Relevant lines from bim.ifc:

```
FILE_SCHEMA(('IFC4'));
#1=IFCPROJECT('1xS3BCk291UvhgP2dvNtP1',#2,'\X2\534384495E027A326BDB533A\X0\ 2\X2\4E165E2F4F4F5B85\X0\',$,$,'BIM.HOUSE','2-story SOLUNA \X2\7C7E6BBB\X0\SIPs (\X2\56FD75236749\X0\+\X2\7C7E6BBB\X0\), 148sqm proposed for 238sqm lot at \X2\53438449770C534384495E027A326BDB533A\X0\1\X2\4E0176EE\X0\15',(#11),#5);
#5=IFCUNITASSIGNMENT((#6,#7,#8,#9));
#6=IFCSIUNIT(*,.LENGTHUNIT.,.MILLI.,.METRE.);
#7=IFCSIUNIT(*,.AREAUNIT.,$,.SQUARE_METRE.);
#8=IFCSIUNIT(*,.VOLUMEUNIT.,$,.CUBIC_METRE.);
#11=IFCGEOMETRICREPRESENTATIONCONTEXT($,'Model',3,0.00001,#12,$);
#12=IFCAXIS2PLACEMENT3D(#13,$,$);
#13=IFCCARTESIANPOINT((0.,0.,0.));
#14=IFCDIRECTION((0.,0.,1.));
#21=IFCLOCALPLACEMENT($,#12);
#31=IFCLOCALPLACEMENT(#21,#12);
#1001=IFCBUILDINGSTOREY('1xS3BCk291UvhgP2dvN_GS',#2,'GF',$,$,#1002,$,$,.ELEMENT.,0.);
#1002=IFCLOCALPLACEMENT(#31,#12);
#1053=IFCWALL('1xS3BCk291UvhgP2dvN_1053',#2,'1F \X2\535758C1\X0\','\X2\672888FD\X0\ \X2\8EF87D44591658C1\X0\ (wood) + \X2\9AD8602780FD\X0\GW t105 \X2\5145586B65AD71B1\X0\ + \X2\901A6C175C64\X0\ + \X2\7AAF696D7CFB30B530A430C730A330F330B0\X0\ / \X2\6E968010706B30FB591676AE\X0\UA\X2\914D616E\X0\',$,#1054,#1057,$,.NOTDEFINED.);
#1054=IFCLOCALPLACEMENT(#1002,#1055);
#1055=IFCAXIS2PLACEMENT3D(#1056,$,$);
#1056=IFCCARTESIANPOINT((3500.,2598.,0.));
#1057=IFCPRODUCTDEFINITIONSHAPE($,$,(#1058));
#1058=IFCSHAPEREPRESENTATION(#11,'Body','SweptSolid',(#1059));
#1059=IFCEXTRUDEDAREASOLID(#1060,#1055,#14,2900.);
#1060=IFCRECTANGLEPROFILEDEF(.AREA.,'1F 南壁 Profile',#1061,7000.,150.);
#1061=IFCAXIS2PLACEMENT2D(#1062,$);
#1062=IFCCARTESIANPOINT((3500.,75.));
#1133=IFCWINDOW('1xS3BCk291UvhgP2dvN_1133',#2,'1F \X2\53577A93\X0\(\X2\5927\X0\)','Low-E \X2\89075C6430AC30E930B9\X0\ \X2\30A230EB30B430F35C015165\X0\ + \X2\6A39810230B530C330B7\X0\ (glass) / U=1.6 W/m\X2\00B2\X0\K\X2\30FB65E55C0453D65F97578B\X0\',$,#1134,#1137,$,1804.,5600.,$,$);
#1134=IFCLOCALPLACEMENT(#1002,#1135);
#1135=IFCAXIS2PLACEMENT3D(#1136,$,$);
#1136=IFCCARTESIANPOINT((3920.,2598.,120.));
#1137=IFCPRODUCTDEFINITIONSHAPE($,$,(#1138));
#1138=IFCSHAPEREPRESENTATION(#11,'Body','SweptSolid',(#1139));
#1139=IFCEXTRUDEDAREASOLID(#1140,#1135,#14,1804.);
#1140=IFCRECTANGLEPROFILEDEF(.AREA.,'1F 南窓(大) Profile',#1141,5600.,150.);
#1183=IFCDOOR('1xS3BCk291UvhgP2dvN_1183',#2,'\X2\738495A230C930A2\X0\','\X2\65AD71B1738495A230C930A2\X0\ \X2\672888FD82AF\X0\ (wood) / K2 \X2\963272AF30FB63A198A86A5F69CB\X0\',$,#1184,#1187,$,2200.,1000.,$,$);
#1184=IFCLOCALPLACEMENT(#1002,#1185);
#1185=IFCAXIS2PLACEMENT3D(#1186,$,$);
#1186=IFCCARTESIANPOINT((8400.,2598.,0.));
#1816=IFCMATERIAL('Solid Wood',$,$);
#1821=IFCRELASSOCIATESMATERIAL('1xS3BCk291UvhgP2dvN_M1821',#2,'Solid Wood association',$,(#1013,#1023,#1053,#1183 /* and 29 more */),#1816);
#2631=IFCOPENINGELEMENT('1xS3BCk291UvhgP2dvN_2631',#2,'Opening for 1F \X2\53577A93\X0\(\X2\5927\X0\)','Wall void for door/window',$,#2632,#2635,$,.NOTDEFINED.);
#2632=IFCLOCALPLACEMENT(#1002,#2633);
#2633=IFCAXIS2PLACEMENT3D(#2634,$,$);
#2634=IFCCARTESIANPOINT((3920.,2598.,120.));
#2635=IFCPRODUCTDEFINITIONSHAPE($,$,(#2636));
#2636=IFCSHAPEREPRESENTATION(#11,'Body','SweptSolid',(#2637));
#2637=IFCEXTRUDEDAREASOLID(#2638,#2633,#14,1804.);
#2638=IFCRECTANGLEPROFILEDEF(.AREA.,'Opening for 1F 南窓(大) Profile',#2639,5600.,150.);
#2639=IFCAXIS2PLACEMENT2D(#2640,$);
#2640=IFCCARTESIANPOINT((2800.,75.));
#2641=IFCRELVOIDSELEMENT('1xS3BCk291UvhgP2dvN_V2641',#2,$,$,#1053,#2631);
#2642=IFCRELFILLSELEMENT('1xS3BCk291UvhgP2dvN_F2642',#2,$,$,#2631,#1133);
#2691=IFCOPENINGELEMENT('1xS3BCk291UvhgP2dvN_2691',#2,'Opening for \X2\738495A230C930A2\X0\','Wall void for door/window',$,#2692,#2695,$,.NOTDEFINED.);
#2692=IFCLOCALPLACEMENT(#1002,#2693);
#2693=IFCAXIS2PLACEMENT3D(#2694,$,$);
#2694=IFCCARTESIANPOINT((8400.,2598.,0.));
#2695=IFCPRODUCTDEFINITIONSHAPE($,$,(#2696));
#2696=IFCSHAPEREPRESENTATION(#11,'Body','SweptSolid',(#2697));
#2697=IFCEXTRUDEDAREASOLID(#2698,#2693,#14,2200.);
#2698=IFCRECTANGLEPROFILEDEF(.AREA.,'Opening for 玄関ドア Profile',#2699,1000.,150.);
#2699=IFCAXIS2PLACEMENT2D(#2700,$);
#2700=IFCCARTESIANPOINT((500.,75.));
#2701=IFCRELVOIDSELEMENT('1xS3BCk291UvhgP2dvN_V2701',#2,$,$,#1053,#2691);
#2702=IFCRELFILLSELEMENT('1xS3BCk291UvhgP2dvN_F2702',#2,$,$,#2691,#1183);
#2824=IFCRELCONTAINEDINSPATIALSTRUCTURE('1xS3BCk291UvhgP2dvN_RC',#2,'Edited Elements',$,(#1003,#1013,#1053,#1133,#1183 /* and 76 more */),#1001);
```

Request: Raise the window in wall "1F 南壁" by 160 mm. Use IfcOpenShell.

```python
import numpy as np
import ifcopenshell
import ifcopenshell.api.geometry
import ifcopenshell.util.placement
import ifcopenshell.util.unit

model = ifcopenshell.open("bim.ifc")
unit_scale = ifcopenshell.util.unit.calculate_unit_scale(model)

window = model.by_guid("1xS3BCk291UvhgP2dvN_1133")
opening = window.FillsVoids[0].RelatingOpeningElement
dz = 0.16 / unit_scale

shift = np.array([0.0, 0.0, dz])
# The window is not placed relative to its opening, so move both.
for product in (opening, window):
    matrix = ifcopenshell.util.placement.get_local_placement(product.ObjectPlacement)
    matrix[:3, 3] += shift
    ifcopenshell.api.geometry.edit_object_placement(model, product=product, matrix=matrix, is_si=False)

print(f"moved by {dz * unit_scale:+.3f} m")

model.write("bim_updated.ifc")
```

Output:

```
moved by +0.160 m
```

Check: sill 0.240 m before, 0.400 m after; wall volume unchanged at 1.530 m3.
